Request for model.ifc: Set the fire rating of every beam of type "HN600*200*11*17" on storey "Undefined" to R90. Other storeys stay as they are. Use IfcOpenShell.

First a look at what the model holds.

```python
import ifcopenshell
import ifcopenshell.util.element

model = ifcopenshell.open("model.ifc")
print(model.schema)
storey = next(s for s in model.by_type("IfcBuildingStorey") if s.Name == "Undefined")
beams = [e for e in ifcopenshell.util.element.get_decomposition(storey) if e.is_a("IfcBeam")]
seen = {}
for e in beams:
    element_type = ifcopenshell.util.element.get_type(e)
    key = (element_type.Name if element_type != e and element_type else None, ifcopenshell.util.element.get_pset(e, "Pset_BeamCommon", "FireRating"))
    seen[key] = seen.get(key, 0) + 1
for (name, value), count in sorted(seen.items(), key=str):
    print(count, "x", name, "|", value)
```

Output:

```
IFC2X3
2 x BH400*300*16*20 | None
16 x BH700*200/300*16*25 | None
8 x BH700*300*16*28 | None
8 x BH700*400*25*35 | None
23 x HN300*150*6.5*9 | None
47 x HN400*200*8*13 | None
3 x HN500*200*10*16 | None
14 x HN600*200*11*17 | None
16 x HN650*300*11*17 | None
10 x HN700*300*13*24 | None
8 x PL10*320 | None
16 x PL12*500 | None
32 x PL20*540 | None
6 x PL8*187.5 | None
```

```python
import ifcopenshell
import ifcopenshell.api.pset
import ifcopenshell.util.element

model = ifcopenshell.open("model.ifc")

storey = next(s for s in model.by_type("IfcBuildingStorey") if s.Name == "Undefined")
beams = [e for e in ifcopenshell.util.element.get_decomposition(storey) if e.is_a("IfcBeam")]

count = 0
for e in beams:
    element_type = ifcopenshell.util.element.get_type(e)
    if element_type in (None, e) or element_type.Name != "HN600*200*11*17":
        continue
    # add_pset returns the element's existing set when there is one.
    pset = ifcopenshell.api.pset.add_pset(model, product=e, name="Pset_BeamCommon")
    ifcopenshell.api.pset.edit_pset(model, pset=pset, properties={"FireRating": "R90"})
    count += 1

print(count, "beams updated")

model.write("model_rev.ifc")
```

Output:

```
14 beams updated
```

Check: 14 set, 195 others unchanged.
